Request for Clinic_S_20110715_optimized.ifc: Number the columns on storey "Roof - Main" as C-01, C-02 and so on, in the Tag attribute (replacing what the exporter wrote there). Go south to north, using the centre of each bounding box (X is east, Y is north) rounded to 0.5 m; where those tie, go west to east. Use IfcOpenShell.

First a look at what the model holds.

```python
import ifcopenshell
import ifcopenshell.util.element
import ifcopenshell.util.placement

model = ifcopenshell.open("Clinic_S_20110715_optimized.ifc")
print(model.schema)
storey = next(s for s in model.by_type("IfcBuildingStorey") if s.Name == "Roof - Main")
columns = [e for e in ifcopenshell.util.element.get_decomposition(storey) if e.is_a("IfcColumn")]
for e in sorted(columns, key=lambda e: e.id()):
    origin = ifcopenshell.util.placement.get_local_placement(e.ObjectPlacement)[:3, 3]
    print(e.id(), e.Tag, e.Name, origin.round(2) + 0.0, sep=" | ")
```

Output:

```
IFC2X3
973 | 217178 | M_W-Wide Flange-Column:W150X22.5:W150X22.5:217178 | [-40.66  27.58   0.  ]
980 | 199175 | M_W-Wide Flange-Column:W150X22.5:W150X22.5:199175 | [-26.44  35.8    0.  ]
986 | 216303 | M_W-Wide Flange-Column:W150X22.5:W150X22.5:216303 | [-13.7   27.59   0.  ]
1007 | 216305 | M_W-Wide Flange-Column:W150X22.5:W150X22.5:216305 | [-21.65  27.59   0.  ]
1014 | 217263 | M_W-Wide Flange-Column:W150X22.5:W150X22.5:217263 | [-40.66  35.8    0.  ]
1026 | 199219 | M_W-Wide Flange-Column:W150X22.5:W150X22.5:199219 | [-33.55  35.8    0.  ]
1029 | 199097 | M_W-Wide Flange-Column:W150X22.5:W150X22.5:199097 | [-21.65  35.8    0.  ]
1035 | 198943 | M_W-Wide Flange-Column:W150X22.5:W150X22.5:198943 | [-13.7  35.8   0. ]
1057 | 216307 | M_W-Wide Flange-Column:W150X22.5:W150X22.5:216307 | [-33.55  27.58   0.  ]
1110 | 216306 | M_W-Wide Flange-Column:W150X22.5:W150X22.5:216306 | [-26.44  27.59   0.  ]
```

```python
import ifcopenshell
import ifcopenshell.geom
import ifcopenshell.util.element
import ifcopenshell.util.shape

model = ifcopenshell.open("Clinic_S_20110715_optimized.ifc")
settings = ifcopenshell.geom.settings()
settings.set("use-world-coords", True)


def centre(element):
    shape = ifcopenshell.geom.create_shape(settings, element)
    return ifcopenshell.util.shape.get_bbox_centroid(shape.geometry)


storey = next(s for s in model.by_type("IfcBuildingStorey") if s.Name == "Roof - Main")
columns = [e for e in ifcopenshell.util.element.get_decomposition(storey) if e.is_a("IfcColumn")]

# Insertion points can sit at a corner or the storey origin, so sort by the geometry (in metres).
centres = {e: centre(e) for e in columns}
columns.sort(key=lambda e: (round(centres[e][1] / 0.5), centres[e][0]))

for i, e in enumerate(columns, start=1):
    number = f"C-{i:02d}"
    e.Tag = number
    print(e.id(), number)

model.write("Clinic_S_20110715_optimized-out.ifc")
```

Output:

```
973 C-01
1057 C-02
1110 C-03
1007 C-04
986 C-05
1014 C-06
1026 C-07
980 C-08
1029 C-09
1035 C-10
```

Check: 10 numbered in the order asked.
